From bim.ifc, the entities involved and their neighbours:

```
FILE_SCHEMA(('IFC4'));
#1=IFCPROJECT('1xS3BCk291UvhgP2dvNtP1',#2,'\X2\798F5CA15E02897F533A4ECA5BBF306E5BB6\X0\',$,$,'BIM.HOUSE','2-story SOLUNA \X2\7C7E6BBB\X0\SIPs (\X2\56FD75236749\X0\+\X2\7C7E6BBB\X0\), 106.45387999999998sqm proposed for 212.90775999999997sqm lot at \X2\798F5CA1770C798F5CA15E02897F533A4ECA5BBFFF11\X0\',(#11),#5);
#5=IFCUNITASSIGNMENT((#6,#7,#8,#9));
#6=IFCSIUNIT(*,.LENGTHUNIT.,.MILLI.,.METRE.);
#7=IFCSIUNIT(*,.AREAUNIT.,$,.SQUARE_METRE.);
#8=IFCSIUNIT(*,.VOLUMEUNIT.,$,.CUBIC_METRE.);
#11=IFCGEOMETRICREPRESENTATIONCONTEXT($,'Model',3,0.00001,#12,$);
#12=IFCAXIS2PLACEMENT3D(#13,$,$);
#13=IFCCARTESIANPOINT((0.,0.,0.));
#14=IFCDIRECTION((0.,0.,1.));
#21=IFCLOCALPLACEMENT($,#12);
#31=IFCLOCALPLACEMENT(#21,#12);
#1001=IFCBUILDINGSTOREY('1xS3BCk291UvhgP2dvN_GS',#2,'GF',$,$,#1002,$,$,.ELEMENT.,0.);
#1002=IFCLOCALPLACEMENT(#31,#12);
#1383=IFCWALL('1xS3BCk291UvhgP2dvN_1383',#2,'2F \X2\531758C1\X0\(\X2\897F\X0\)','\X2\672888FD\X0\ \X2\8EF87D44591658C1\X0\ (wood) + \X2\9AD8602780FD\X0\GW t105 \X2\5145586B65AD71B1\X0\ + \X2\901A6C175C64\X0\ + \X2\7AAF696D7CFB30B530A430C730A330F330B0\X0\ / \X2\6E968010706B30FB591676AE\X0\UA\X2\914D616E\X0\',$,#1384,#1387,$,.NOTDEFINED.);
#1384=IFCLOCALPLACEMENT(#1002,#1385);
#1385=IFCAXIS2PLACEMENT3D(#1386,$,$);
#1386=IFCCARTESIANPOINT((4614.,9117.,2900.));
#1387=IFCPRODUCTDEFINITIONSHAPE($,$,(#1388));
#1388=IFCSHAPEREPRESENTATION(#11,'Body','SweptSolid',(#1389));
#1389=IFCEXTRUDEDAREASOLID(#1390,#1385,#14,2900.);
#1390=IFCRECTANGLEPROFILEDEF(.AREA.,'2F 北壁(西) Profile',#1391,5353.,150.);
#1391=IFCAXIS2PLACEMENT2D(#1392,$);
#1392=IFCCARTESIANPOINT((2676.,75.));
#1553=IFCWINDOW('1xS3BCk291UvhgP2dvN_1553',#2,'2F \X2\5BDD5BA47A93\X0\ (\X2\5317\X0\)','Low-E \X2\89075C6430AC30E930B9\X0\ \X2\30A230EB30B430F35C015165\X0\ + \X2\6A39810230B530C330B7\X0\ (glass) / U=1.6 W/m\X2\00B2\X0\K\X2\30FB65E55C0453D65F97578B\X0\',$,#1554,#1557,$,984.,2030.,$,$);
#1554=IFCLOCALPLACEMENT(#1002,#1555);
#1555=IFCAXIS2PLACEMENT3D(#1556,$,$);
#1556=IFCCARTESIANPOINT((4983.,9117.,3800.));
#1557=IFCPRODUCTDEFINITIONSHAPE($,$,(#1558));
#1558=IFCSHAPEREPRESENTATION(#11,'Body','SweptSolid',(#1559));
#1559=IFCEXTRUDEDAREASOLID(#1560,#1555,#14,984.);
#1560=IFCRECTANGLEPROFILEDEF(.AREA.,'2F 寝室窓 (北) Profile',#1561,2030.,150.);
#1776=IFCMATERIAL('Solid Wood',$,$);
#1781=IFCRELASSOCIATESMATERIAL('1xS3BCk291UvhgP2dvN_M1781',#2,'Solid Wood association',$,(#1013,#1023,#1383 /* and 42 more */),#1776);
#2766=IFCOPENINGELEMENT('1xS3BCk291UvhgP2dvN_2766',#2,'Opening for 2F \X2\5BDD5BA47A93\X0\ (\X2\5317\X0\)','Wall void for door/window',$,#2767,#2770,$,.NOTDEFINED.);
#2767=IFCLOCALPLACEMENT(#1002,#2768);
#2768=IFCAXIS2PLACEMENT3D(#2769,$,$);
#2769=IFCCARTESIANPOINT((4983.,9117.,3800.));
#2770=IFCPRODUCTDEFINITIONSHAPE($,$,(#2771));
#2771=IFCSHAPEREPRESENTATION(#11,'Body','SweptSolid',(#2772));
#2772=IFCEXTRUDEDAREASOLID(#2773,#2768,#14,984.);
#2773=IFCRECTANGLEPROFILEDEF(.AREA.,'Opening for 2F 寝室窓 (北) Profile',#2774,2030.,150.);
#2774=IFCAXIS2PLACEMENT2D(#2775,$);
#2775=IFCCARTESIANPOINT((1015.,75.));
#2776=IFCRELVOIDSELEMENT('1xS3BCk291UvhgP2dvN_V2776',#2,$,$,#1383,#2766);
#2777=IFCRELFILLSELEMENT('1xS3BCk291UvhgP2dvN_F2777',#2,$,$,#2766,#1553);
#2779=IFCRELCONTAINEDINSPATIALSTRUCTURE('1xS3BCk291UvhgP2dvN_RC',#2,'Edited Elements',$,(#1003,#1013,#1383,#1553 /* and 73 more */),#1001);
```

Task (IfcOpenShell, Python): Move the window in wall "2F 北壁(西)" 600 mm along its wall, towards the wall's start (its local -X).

```python
import ifcopenshell
import ifcopenshell.api.geometry
import ifcopenshell.util.placement
import ifcopenshell.util.unit

model = ifcopenshell.open("bim.ifc")
unit_scale = ifcopenshell.util.unit.calculate_unit_scale(model)

window = model.by_id(1553)
opening = window.FillsVoids[0].RelatingOpeningElement
wall = opening.VoidsElements[0].RelatingBuildingElement

wall_matrix = ifcopenshell.util.placement.get_local_placement(wall.ObjectPlacement)
shift = wall_matrix[:3, 0] * -0.6 / unit_scale
before = ifcopenshell.util.placement.get_local_placement(window.ObjectPlacement)[:3, 3].copy()

# The window is not placed relative to its opening, so move both.
for product in (opening, window):
    matrix = ifcopenshell.util.placement.get_local_placement(product.ObjectPlacement)
    matrix[:3, 3] += shift
    ifcopenshell.api.geometry.edit_object_placement(model, product=product, matrix=matrix, is_si=False)

after = ifcopenshell.util.placement.get_local_placement(window.ObjectPlacement)[:3, 3]
print("window moved by", (after - before).round(3) + 0.0)

model.write("bim_v2.ifc")
```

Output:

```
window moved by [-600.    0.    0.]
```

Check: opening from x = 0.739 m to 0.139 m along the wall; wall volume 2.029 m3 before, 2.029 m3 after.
